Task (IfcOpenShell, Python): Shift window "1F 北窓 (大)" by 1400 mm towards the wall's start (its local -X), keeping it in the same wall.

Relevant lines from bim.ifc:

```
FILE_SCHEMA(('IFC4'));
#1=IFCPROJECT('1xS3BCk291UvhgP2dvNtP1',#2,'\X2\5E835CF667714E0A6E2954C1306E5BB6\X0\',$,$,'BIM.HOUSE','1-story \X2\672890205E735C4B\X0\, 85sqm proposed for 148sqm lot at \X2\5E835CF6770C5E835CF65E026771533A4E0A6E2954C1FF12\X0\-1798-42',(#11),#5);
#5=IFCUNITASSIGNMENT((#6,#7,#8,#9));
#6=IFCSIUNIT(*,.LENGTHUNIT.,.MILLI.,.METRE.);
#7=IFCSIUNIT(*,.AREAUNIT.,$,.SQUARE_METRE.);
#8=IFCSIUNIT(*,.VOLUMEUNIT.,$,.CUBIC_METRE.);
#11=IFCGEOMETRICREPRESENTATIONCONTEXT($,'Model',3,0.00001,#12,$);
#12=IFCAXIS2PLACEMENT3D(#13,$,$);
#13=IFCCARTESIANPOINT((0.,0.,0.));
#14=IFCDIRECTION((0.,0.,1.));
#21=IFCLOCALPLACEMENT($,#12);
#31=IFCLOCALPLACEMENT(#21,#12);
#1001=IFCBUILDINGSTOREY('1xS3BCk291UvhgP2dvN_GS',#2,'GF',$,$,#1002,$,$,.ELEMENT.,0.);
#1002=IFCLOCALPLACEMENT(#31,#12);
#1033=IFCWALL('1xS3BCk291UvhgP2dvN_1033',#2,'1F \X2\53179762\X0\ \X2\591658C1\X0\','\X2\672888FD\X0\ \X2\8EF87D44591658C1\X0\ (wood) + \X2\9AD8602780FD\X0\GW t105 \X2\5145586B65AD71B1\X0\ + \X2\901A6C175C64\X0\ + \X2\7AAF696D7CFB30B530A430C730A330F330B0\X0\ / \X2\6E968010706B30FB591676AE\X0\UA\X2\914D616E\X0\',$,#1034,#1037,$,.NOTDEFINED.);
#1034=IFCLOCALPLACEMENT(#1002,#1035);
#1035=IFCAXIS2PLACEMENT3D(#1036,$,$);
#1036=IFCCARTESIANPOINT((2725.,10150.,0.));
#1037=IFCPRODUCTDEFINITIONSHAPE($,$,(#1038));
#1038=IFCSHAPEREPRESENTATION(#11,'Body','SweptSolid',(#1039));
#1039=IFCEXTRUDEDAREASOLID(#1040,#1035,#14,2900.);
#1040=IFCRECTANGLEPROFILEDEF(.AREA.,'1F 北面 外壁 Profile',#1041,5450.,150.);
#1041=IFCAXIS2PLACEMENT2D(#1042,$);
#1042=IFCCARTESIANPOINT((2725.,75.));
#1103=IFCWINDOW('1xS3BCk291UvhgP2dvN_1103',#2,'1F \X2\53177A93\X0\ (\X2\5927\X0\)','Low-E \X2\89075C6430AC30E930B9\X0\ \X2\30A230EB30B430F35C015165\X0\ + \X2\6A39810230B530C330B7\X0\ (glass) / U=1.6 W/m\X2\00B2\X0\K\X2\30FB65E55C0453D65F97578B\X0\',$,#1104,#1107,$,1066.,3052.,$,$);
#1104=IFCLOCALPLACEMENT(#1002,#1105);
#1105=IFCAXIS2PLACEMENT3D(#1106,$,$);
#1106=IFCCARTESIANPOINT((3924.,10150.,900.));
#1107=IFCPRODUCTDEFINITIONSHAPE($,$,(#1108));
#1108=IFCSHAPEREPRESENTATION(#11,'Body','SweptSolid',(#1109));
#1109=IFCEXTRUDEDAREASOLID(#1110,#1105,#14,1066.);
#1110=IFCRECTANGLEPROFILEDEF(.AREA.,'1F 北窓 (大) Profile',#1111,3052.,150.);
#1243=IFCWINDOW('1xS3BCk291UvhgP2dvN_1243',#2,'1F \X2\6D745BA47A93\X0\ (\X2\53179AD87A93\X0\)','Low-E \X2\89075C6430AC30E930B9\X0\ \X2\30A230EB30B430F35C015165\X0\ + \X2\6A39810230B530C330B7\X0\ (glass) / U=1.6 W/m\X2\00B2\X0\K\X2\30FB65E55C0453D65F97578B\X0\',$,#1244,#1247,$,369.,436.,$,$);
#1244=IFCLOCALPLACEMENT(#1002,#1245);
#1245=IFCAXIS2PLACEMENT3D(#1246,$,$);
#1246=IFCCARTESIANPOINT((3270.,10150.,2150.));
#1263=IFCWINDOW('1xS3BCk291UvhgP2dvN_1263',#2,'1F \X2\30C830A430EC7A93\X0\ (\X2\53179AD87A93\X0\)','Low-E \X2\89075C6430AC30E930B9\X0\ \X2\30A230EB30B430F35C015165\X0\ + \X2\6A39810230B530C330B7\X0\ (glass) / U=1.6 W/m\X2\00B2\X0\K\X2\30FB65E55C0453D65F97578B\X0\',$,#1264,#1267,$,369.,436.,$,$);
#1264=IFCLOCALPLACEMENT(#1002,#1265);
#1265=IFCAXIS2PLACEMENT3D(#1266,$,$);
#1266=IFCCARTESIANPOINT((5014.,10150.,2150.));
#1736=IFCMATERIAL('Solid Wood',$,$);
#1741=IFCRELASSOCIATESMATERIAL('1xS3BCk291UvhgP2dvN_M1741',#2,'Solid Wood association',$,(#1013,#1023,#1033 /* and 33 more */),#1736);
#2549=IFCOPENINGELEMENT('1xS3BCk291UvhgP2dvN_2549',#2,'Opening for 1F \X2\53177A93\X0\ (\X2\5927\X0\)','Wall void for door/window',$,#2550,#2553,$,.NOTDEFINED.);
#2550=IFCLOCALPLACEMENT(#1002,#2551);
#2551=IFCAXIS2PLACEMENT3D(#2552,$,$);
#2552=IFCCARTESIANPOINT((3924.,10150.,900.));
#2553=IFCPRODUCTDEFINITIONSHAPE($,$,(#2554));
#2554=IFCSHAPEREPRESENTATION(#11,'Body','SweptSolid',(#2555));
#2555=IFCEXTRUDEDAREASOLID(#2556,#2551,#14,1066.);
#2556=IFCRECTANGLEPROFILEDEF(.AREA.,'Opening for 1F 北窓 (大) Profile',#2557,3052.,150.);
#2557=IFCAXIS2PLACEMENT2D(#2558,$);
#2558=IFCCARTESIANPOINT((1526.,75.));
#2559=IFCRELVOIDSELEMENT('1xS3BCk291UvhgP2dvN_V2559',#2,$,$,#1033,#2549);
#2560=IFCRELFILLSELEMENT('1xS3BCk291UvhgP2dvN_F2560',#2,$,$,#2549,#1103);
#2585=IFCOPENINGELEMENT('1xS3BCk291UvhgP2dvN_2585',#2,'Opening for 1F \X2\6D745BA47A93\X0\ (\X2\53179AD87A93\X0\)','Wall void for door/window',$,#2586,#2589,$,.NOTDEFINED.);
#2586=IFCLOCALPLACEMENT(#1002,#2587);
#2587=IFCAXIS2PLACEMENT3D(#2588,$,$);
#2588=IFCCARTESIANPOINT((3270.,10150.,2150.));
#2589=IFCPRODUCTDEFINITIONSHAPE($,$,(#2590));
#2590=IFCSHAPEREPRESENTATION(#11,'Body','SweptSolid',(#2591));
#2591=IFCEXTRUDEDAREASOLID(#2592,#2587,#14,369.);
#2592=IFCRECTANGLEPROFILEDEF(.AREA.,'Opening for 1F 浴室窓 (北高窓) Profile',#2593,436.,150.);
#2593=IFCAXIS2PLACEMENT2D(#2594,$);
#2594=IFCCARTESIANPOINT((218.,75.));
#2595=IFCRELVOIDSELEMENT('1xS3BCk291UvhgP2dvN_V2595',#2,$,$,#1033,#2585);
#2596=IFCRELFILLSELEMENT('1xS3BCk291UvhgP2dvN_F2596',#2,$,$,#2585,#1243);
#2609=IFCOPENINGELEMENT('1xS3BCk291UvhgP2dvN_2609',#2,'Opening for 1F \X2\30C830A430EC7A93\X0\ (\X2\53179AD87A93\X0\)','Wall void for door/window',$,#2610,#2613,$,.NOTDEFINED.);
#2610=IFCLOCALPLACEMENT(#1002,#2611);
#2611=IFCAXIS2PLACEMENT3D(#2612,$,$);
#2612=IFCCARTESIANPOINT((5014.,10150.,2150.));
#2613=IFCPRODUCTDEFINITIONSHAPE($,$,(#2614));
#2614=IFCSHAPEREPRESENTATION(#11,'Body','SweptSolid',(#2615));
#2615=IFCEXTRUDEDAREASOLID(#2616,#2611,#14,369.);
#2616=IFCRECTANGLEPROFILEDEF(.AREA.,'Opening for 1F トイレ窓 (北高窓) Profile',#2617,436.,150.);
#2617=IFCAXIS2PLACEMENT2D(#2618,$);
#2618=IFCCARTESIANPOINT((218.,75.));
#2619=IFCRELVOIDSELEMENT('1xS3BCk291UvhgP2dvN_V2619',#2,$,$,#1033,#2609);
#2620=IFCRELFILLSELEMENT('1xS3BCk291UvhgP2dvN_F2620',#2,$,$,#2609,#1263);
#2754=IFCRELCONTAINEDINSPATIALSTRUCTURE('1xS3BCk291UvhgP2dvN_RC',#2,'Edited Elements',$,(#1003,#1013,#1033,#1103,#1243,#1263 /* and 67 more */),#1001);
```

```python
import ifcopenshell
import ifcopenshell.api.geometry
import ifcopenshell.util.placement

model = ifcopenshell.open("bim.ifc")

window = model.by_guid("1xS3BCk291UvhgP2dvN_1103")
opening = window.FillsVoids[0].RelatingOpeningElement
wall = opening.VoidsElements[0].RelatingBuildingElement

wall_matrix = ifcopenshell.util.placement.get_local_placement(wall.ObjectPlacement)
shift = wall_matrix[:3, 0] * -1400.0
before = ifcopenshell.util.placement.get_local_placement(window.ObjectPlacement)[:3, 3].copy()

# The window is not placed relative to its opening, so move both.
for product in (opening, window):
    matrix = ifcopenshell.util.placement.get_local_placement(product.ObjectPlacement)
    matrix[:3, 3] += shift
    ifcopenshell.api.geometry.edit_object_placement(model, product=product, matrix=matrix, is_si=False)

after = ifcopenshell.util.placement.get_local_placement(window.ObjectPlacement)[:3, 3]
print("window moved by", (after - before).round(3) + 0.0)

model.write("bim_v2.ifc")
```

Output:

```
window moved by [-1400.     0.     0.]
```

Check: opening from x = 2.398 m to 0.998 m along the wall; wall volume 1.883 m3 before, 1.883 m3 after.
